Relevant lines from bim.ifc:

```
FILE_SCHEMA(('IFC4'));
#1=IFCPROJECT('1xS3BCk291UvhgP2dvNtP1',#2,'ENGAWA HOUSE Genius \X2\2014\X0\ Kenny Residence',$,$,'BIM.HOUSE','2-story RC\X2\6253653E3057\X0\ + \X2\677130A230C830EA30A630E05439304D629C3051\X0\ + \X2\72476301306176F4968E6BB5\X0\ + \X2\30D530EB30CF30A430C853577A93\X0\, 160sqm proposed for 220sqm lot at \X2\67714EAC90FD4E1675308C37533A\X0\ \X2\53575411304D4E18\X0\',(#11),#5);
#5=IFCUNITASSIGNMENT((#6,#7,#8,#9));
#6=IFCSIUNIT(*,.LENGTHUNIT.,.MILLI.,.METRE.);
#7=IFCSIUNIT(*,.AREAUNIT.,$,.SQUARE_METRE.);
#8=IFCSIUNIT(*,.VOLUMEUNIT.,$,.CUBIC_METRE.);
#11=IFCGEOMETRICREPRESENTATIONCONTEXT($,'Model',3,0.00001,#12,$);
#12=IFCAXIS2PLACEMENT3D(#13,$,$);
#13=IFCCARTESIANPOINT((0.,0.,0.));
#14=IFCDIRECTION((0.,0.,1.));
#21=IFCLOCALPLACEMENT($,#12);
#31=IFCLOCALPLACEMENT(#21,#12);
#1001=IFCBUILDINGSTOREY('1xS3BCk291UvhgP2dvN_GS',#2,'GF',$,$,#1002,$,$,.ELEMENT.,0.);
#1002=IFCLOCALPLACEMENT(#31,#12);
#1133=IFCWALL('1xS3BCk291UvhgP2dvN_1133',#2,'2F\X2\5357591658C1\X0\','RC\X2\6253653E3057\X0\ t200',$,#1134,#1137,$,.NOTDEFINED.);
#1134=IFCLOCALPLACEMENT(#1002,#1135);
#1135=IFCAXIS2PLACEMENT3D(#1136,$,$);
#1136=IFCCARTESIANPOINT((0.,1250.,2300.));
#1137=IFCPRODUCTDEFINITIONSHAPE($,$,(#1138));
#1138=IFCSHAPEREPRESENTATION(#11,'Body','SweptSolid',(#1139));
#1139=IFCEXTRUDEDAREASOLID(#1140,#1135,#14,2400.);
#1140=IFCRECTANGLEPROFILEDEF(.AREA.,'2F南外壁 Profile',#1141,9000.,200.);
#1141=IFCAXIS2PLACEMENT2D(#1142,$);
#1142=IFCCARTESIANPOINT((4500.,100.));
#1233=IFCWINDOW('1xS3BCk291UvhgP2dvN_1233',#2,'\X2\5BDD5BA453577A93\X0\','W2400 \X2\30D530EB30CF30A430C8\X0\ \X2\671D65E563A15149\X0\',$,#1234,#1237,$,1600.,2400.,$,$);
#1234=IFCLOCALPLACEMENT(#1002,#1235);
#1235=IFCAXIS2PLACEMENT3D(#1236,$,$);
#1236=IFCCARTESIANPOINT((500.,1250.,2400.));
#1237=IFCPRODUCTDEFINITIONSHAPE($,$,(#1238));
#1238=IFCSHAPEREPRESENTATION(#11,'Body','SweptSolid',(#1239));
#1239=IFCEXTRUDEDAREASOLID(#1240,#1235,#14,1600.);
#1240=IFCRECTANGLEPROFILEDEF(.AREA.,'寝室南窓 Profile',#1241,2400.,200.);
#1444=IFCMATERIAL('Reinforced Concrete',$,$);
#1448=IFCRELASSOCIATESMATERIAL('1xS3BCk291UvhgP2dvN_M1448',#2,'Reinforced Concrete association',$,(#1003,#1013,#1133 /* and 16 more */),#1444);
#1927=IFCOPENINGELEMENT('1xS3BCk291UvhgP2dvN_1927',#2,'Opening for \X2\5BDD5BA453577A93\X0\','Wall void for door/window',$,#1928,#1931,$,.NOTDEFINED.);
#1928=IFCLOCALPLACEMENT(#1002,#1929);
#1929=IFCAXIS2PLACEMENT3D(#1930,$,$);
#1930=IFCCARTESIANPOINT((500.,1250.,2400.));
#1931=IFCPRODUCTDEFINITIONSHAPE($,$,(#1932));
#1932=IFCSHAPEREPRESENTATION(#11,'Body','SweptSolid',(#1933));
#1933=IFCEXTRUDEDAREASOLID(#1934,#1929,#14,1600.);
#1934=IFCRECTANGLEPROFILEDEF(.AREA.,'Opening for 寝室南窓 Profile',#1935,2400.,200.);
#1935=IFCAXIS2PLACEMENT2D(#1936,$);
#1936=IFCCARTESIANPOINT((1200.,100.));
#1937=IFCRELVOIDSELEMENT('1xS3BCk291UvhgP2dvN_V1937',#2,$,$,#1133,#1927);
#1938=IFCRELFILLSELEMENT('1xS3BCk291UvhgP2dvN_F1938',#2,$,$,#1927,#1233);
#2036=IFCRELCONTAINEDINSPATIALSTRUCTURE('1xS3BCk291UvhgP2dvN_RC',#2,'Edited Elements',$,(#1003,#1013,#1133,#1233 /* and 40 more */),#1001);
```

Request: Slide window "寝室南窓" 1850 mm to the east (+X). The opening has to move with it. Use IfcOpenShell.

```python
import ifcopenshell
import ifcopenshell.api.geometry
import ifcopenshell.util.placement
import ifcopenshell.util.unit

model = ifcopenshell.open("bim.ifc")
unit_scale = ifcopenshell.util.unit.calculate_unit_scale(model)

window = model.by_id(1233)
opening = window.FillsVoids[0].RelatingOpeningElement
wall = opening.VoidsElements[0].RelatingBuildingElement

wall_matrix = ifcopenshell.util.placement.get_local_placement(wall.ObjectPlacement)
shift = wall_matrix[:3, 0] * 1.85 / unit_scale
before = ifcopenshell.util.placement.get_local_placement(window.ObjectPlacement)[:3, 3].copy()

# The window is not placed relative to its opening, so move both.
for product in (opening, window):
    matrix = ifcopenshell.util.placement.get_local_placement(product.ObjectPlacement)
    matrix[:3, 3] += shift
    ifcopenshell.api.geometry.edit_object_placement(model, product=product, matrix=matrix, is_si=False)

after = ifcopenshell.util.placement.get_local_placement(window.ObjectPlacement)[:3, 3]
print("window moved by", (after - before).round(3) + 0.0)

model.write("bim_edited.ifc")
```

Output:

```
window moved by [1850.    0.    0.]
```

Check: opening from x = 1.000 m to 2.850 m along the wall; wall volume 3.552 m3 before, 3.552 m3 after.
